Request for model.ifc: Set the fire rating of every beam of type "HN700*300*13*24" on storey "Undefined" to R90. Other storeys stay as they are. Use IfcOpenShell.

First a look at what the model holds.

```python
import ifcopenshell
import ifcopenshell.util.element

model = ifcopenshell.open("model.ifc")
print(model.schema)
storey = next(s for s in model.by_type("IfcBuildingStorey") if s.Name == "Undefined")
beams = [e for e in ifcopenshell.util.element.get_decomposition(storey) if e.is_a("IfcBeam")]
seen = {}
for e in beams:
    element_type = ifcopenshell.util.element.get_type(e)
    key = (element_type.Name if element_type != e and element_type else None, ifcopenshell.util.element.get_pset(e, "Pset_BeamCommon", "FireRating"))
    seen[key] = seen.get(key, 0) + 1
for (name, value), count in sorted(seen.items(), key=str):
    print(count, "x", name, "|", value)
```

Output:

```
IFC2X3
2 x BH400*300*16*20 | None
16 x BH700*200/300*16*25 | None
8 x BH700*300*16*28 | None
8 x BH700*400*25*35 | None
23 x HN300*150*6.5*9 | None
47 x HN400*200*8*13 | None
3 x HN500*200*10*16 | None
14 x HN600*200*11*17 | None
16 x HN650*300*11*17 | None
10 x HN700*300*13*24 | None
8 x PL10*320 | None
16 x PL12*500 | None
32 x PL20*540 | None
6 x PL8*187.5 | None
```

```python
import ifcopenshell
import ifcopenshell.api.pset
import ifcopenshell.util.element

model = ifcopenshell.open("model.ifc")

storey = next(s for s in model.by_type("IfcBuildingStorey") if s.Name == "Undefined")
beams = [e for e in ifcopenshell.util.element.get_decomposition(storey) if e.is_a("IfcBeam")]

count = 0
for e in beams:
    element_type = ifcopenshell.util.element.get_type(e)
    if element_type in (None, e) or element_type.Name != "HN700*300*13*24":
        continue
    # add_pset returns the element's existing set when there is one.
    pset = ifcopenshell.api.pset.add_pset(model, product=e, name="Pset_BeamCommon")
    ifcopenshell.api.pset.edit_pset(model, pset=pset, properties={"FireRating": "R90"})
    count += 1

print(count, "beams updated")

model.write("model_rev.ifc")
```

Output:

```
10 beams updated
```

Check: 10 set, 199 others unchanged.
